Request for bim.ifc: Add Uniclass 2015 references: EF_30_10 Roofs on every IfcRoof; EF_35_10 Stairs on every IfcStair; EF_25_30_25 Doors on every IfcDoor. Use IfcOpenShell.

First a look at what the model holds.

```python
import ifcopenshell

model = ifcopenshell.open("bim.ifc")
print(model.schema)
print("classifications:", [c.Name for c in model.by_type("IfcClassification")])
for ifc_class in ("IfcDoor", "IfcRoof", "IfcStair", "IfcWall", "IfcWindow"):
    print(ifc_class, len(model.by_type(ifc_class)))
```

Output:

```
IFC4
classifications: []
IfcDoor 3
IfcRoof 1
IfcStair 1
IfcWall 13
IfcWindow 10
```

```python
import ifcopenshell
import ifcopenshell.api.classification

model = ifcopenshell.open("bim.ifc")

system = ifcopenshell.api.classification.add_classification(model, classification="Uniclass 2015")

codes = {
    "IfcRoof": ("EF_30_10", "Roofs"),
    "IfcStair": ("EF_35_10", "Stairs"),
    "IfcDoor": ("EF_25_30_25", "Doors"),
}
for ifc_class, (code, name) in codes.items():
    products = model.by_type(ifc_class)
    ifcopenshell.api.classification.add_reference(
        model, products=products, classification=system, identification=code, name=name
    )
    print(code, len(products))

model.write("bim_v2.ifc")
```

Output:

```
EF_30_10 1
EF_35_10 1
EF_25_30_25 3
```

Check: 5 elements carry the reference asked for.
